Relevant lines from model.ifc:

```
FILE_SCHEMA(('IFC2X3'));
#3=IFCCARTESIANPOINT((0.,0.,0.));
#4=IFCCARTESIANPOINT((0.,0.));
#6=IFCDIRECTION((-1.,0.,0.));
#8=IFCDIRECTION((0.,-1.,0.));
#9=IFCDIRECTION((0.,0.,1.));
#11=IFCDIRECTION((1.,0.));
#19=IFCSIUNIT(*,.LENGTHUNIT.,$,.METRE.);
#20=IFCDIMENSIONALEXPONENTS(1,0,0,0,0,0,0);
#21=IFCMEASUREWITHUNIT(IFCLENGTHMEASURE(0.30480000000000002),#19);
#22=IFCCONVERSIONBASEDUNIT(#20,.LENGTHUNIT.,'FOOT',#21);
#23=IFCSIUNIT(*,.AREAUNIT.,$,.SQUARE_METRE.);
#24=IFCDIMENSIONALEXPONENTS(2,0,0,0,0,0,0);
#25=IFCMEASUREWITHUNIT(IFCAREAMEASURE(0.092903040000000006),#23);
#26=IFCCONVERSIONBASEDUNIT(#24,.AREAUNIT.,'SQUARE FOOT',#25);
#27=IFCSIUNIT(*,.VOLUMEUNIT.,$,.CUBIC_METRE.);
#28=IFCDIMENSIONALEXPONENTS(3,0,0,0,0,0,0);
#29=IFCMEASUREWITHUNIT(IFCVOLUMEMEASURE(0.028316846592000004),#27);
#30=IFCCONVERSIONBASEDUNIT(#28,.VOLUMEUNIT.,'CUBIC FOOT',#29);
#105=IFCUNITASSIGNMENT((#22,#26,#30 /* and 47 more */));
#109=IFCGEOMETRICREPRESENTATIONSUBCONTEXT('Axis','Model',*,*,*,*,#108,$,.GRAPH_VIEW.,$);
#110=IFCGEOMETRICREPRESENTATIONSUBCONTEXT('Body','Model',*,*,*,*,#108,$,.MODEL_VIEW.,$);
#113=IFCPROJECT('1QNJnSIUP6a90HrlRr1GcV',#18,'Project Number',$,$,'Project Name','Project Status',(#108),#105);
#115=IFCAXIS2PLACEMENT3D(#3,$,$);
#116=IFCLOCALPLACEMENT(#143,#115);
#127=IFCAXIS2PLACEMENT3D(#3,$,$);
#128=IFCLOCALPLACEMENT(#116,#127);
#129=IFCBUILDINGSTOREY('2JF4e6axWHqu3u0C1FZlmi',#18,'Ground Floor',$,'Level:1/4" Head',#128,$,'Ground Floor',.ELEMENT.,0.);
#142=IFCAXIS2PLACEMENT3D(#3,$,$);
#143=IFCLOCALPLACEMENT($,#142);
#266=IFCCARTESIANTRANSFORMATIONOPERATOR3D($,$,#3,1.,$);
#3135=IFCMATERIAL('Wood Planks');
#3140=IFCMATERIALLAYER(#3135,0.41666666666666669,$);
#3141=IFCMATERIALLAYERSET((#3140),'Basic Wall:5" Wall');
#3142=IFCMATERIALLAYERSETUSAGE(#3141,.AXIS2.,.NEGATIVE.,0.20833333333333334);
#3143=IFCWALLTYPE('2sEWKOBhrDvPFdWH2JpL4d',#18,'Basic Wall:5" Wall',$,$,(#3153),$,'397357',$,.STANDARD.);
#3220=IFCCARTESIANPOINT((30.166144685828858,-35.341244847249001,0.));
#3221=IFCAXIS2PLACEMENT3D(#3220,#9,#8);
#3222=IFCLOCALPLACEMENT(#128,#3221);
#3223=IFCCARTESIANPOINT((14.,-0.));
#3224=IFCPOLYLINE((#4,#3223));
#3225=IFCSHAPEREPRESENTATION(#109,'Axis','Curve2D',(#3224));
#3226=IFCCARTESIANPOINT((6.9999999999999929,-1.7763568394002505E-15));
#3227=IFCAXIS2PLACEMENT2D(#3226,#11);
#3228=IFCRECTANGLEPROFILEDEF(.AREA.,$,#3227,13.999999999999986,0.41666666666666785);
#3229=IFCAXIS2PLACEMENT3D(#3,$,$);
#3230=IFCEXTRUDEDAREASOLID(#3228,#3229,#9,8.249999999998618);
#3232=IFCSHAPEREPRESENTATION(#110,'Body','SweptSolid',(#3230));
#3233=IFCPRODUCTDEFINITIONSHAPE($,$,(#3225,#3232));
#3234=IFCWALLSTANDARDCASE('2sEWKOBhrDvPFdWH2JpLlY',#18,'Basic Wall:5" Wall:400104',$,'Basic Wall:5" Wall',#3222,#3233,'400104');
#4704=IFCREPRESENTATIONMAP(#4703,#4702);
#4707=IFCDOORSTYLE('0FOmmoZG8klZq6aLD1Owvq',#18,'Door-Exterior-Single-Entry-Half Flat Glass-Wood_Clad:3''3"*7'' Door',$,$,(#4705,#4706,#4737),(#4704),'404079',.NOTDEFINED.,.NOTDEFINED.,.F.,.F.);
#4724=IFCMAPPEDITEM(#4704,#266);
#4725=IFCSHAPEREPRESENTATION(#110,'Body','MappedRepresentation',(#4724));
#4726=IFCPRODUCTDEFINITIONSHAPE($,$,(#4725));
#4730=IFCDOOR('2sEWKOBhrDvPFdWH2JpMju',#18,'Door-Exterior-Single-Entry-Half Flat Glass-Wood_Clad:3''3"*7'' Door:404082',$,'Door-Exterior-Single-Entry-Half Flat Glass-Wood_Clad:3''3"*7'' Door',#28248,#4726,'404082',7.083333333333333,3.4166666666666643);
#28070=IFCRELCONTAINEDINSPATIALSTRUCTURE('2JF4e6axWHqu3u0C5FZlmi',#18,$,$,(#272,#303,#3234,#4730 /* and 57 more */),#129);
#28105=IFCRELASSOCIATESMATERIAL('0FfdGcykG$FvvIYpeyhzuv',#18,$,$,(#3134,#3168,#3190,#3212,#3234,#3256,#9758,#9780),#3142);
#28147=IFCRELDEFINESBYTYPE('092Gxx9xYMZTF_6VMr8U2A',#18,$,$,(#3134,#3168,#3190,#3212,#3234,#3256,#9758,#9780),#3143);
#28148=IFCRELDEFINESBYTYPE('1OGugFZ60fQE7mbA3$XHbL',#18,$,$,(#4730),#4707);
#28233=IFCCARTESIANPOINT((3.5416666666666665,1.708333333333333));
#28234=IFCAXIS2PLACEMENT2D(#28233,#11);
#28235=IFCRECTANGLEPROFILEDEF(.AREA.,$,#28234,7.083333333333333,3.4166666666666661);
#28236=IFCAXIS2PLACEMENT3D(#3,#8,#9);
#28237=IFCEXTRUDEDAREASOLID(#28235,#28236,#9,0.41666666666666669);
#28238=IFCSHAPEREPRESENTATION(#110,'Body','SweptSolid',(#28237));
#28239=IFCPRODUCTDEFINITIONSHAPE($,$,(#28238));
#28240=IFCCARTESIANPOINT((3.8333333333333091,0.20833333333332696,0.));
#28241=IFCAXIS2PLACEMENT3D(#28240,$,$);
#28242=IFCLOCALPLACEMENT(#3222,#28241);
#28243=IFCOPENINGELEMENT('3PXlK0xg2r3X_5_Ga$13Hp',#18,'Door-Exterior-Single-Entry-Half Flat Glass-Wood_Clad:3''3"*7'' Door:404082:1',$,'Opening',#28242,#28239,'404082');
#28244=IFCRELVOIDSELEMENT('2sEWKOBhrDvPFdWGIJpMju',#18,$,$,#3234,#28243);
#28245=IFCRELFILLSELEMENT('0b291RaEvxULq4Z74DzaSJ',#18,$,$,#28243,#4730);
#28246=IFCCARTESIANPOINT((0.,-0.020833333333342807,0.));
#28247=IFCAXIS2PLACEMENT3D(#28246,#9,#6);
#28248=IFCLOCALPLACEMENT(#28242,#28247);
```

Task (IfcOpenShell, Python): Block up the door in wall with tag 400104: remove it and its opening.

```python
import ifcopenshell
import ifcopenshell.api.feature
import ifcopenshell.api.root
import ifcopenshell.geom
import ifcopenshell.util.shape

model = ifcopenshell.open("model.ifc")
settings = ifcopenshell.geom.settings()


def volume(element):
    """Net volume in cubic metres, openings subtracted."""
    shape = ifcopenshell.geom.create_shape(settings, element)
    return ifcopenshell.util.shape.get_volume(shape.geometry)


door = model.by_guid("2sEWKOBhrDvPFdWH2JpMju")
opening = door.FillsVoids[0].RelatingOpeningElement
wall = opening.VoidsElements[0].RelatingBuildingElement
before = volume(wall)

ifcopenshell.api.root.remove_product(model, product=door)
ifcopenshell.api.feature.remove_feature(model, feature=opening)

after = volume(wall)

print(f"wall volume {before:.3f} -> {after:.3f} m3")

model.write("model_edited.ifc")
```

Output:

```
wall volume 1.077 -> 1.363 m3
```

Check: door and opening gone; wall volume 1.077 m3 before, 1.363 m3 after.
